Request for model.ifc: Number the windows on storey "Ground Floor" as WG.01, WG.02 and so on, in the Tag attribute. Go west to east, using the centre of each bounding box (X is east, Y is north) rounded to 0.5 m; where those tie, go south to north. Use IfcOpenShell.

First a look at what the model holds.

```python
import ifcopenshell
import ifcopenshell.util.element
import ifcopenshell.util.placement

model = ifcopenshell.open("model.ifc")
print(model.schema)
storey = next(s for s in model.by_type("IfcBuildingStorey") if s.Name == "Ground Floor")
windows = [e for e in ifcopenshell.util.element.get_decomposition(storey) if e.is_a("IfcWindow")]
for e in sorted(windows, key=lambda e: e.id()):
    origin = ifcopenshell.util.placement.get_local_placement(e.ObjectPlacement)[:3, 3]
    print(e.id(), e.Tag, e.Name, origin.round(2) + 0.0, sep=" | ")
```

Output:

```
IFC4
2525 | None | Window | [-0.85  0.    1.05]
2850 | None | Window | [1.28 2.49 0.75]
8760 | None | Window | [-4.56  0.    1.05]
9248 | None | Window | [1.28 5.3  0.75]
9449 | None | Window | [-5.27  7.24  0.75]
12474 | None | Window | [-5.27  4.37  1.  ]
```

```python
import ifcopenshell
import ifcopenshell.geom
import ifcopenshell.util.element
import ifcopenshell.util.shape

model = ifcopenshell.open("model.ifc")
settings = ifcopenshell.geom.settings()
settings.set("use-world-coords", True)


def centre(element):
    shape = ifcopenshell.geom.create_shape(settings, element)
    return ifcopenshell.util.shape.get_bbox_centroid(shape.geometry)


storey = next(s for s in model.by_type("IfcBuildingStorey") if s.Name == "Ground Floor")
windows = [e for e in ifcopenshell.util.element.get_decomposition(storey) if e.is_a("IfcWindow")]

# Insertion points can sit at a corner or the storey origin, so sort by the geometry (in metres).
centres = {e: centre(e) for e in windows}
windows.sort(key=lambda e: (round(centres[e][0] / 0.5), centres[e][1]))

for i, e in enumerate(windows, start=1):
    number = f"WG.{i:02d}"
    e.Tag = number
    print(e.id(), number)

model.write("model-out.ifc")
```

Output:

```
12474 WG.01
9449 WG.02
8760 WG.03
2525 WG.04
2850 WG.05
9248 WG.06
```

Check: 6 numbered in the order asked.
